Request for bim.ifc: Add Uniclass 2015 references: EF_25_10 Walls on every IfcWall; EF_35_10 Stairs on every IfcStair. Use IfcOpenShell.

First a look at what the model holds.

```python
import ifcopenshell

model = ifcopenshell.open("bim.ifc")
print(model.schema)
print("classifications:", [c.Name for c in model.by_type("IfcClassification")])
for ifc_class in ("IfcDoor", "IfcRoof", "IfcStair", "IfcWall", "IfcWindow"):
    print(ifc_class, len(model.by_type(ifc_class)))
```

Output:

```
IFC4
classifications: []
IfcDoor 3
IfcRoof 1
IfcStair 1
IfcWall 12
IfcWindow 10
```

```python
import ifcopenshell
import ifcopenshell.api.classification

model = ifcopenshell.open("bim.ifc")

system = ifcopenshell.api.classification.add_classification(model, classification="Uniclass 2015")

codes = {
    "IfcWall": ("EF_25_10", "Walls"),
    "IfcStair": ("EF_35_10", "Stairs"),
}
for ifc_class, (code, name) in codes.items():
    products = model.by_type(ifc_class)
    ifcopenshell.api.classification.add_reference(
        model, products=products, classification=system, identification=code, name=name
    )
    print(code, len(products))

model.write("bim_updated.ifc")
```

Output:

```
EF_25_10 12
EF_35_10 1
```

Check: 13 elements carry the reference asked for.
